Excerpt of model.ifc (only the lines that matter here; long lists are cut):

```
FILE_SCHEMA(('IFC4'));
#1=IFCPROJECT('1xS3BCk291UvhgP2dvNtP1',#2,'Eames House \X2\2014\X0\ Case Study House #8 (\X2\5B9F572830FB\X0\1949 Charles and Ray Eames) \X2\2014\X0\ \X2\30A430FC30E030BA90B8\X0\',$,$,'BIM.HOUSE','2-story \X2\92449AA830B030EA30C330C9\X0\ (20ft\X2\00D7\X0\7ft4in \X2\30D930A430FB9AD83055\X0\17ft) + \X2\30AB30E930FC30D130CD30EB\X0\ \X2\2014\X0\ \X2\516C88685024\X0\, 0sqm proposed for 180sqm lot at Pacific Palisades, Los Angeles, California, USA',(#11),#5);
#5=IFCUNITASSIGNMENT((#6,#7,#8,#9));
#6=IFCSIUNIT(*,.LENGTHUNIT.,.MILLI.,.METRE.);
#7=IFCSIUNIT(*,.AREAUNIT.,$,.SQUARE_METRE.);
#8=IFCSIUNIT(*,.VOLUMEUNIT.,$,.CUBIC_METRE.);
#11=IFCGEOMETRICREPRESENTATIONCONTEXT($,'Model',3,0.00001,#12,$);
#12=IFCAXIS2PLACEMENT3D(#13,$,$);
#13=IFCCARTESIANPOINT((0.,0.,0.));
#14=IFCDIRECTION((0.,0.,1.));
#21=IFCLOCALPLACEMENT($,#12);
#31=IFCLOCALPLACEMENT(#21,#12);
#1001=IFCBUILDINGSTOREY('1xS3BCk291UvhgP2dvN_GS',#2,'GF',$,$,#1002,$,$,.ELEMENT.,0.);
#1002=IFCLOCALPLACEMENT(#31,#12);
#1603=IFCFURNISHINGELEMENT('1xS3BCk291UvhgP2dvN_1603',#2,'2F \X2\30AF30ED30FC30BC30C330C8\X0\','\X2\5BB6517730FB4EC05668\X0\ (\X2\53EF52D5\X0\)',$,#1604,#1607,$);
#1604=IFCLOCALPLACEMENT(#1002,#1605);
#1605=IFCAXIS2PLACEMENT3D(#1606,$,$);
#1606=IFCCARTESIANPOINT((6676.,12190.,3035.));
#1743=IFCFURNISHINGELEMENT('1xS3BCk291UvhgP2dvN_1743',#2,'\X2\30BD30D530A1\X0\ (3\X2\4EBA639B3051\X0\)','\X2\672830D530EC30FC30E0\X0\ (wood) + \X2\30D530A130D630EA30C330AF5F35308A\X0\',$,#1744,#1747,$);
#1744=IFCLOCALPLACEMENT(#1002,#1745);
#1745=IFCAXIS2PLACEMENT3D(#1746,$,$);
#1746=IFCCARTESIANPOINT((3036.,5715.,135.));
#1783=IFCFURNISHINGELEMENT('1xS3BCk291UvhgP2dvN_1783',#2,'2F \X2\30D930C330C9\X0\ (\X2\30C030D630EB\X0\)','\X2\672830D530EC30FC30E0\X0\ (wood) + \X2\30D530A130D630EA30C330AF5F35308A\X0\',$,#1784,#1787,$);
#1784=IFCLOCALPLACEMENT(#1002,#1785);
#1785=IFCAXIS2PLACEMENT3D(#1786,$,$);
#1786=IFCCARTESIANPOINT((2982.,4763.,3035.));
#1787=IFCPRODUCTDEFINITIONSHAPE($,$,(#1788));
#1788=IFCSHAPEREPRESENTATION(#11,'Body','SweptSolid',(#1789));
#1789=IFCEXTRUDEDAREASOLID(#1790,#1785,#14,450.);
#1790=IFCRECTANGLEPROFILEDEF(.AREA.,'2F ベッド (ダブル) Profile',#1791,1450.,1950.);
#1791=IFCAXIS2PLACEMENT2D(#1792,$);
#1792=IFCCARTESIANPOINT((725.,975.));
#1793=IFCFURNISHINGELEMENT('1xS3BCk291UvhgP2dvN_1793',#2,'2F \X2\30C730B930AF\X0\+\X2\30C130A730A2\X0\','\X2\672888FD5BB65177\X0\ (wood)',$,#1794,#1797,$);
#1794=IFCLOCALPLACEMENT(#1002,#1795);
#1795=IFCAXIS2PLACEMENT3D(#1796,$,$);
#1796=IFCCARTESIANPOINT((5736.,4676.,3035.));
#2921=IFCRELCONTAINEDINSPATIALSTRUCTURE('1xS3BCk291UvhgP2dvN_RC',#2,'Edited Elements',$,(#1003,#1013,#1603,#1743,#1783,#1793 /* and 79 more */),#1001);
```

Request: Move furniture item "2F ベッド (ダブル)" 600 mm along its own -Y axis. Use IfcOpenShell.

```python
import ifcopenshell
import ifcopenshell.api.geometry
import ifcopenshell.util.placement

model = ifcopenshell.open("model.ifc")

item = model.by_guid("1xS3BCk291UvhgP2dvN_1783")
matrix = ifcopenshell.util.placement.get_local_placement(item.ObjectPlacement)
matrix[:3, 3] -= matrix[:3, 1] * 600.0
ifcopenshell.api.geometry.edit_object_placement(model, product=item, matrix=matrix, is_si=False)

print(ifcopenshell.util.placement.get_local_placement(item.ObjectPlacement).round(3) + 0.0)

model.write("model_edited.ifc")
```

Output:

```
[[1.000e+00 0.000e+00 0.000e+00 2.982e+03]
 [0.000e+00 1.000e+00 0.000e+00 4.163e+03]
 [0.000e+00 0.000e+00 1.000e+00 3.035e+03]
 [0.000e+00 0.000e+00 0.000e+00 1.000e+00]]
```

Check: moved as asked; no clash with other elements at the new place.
